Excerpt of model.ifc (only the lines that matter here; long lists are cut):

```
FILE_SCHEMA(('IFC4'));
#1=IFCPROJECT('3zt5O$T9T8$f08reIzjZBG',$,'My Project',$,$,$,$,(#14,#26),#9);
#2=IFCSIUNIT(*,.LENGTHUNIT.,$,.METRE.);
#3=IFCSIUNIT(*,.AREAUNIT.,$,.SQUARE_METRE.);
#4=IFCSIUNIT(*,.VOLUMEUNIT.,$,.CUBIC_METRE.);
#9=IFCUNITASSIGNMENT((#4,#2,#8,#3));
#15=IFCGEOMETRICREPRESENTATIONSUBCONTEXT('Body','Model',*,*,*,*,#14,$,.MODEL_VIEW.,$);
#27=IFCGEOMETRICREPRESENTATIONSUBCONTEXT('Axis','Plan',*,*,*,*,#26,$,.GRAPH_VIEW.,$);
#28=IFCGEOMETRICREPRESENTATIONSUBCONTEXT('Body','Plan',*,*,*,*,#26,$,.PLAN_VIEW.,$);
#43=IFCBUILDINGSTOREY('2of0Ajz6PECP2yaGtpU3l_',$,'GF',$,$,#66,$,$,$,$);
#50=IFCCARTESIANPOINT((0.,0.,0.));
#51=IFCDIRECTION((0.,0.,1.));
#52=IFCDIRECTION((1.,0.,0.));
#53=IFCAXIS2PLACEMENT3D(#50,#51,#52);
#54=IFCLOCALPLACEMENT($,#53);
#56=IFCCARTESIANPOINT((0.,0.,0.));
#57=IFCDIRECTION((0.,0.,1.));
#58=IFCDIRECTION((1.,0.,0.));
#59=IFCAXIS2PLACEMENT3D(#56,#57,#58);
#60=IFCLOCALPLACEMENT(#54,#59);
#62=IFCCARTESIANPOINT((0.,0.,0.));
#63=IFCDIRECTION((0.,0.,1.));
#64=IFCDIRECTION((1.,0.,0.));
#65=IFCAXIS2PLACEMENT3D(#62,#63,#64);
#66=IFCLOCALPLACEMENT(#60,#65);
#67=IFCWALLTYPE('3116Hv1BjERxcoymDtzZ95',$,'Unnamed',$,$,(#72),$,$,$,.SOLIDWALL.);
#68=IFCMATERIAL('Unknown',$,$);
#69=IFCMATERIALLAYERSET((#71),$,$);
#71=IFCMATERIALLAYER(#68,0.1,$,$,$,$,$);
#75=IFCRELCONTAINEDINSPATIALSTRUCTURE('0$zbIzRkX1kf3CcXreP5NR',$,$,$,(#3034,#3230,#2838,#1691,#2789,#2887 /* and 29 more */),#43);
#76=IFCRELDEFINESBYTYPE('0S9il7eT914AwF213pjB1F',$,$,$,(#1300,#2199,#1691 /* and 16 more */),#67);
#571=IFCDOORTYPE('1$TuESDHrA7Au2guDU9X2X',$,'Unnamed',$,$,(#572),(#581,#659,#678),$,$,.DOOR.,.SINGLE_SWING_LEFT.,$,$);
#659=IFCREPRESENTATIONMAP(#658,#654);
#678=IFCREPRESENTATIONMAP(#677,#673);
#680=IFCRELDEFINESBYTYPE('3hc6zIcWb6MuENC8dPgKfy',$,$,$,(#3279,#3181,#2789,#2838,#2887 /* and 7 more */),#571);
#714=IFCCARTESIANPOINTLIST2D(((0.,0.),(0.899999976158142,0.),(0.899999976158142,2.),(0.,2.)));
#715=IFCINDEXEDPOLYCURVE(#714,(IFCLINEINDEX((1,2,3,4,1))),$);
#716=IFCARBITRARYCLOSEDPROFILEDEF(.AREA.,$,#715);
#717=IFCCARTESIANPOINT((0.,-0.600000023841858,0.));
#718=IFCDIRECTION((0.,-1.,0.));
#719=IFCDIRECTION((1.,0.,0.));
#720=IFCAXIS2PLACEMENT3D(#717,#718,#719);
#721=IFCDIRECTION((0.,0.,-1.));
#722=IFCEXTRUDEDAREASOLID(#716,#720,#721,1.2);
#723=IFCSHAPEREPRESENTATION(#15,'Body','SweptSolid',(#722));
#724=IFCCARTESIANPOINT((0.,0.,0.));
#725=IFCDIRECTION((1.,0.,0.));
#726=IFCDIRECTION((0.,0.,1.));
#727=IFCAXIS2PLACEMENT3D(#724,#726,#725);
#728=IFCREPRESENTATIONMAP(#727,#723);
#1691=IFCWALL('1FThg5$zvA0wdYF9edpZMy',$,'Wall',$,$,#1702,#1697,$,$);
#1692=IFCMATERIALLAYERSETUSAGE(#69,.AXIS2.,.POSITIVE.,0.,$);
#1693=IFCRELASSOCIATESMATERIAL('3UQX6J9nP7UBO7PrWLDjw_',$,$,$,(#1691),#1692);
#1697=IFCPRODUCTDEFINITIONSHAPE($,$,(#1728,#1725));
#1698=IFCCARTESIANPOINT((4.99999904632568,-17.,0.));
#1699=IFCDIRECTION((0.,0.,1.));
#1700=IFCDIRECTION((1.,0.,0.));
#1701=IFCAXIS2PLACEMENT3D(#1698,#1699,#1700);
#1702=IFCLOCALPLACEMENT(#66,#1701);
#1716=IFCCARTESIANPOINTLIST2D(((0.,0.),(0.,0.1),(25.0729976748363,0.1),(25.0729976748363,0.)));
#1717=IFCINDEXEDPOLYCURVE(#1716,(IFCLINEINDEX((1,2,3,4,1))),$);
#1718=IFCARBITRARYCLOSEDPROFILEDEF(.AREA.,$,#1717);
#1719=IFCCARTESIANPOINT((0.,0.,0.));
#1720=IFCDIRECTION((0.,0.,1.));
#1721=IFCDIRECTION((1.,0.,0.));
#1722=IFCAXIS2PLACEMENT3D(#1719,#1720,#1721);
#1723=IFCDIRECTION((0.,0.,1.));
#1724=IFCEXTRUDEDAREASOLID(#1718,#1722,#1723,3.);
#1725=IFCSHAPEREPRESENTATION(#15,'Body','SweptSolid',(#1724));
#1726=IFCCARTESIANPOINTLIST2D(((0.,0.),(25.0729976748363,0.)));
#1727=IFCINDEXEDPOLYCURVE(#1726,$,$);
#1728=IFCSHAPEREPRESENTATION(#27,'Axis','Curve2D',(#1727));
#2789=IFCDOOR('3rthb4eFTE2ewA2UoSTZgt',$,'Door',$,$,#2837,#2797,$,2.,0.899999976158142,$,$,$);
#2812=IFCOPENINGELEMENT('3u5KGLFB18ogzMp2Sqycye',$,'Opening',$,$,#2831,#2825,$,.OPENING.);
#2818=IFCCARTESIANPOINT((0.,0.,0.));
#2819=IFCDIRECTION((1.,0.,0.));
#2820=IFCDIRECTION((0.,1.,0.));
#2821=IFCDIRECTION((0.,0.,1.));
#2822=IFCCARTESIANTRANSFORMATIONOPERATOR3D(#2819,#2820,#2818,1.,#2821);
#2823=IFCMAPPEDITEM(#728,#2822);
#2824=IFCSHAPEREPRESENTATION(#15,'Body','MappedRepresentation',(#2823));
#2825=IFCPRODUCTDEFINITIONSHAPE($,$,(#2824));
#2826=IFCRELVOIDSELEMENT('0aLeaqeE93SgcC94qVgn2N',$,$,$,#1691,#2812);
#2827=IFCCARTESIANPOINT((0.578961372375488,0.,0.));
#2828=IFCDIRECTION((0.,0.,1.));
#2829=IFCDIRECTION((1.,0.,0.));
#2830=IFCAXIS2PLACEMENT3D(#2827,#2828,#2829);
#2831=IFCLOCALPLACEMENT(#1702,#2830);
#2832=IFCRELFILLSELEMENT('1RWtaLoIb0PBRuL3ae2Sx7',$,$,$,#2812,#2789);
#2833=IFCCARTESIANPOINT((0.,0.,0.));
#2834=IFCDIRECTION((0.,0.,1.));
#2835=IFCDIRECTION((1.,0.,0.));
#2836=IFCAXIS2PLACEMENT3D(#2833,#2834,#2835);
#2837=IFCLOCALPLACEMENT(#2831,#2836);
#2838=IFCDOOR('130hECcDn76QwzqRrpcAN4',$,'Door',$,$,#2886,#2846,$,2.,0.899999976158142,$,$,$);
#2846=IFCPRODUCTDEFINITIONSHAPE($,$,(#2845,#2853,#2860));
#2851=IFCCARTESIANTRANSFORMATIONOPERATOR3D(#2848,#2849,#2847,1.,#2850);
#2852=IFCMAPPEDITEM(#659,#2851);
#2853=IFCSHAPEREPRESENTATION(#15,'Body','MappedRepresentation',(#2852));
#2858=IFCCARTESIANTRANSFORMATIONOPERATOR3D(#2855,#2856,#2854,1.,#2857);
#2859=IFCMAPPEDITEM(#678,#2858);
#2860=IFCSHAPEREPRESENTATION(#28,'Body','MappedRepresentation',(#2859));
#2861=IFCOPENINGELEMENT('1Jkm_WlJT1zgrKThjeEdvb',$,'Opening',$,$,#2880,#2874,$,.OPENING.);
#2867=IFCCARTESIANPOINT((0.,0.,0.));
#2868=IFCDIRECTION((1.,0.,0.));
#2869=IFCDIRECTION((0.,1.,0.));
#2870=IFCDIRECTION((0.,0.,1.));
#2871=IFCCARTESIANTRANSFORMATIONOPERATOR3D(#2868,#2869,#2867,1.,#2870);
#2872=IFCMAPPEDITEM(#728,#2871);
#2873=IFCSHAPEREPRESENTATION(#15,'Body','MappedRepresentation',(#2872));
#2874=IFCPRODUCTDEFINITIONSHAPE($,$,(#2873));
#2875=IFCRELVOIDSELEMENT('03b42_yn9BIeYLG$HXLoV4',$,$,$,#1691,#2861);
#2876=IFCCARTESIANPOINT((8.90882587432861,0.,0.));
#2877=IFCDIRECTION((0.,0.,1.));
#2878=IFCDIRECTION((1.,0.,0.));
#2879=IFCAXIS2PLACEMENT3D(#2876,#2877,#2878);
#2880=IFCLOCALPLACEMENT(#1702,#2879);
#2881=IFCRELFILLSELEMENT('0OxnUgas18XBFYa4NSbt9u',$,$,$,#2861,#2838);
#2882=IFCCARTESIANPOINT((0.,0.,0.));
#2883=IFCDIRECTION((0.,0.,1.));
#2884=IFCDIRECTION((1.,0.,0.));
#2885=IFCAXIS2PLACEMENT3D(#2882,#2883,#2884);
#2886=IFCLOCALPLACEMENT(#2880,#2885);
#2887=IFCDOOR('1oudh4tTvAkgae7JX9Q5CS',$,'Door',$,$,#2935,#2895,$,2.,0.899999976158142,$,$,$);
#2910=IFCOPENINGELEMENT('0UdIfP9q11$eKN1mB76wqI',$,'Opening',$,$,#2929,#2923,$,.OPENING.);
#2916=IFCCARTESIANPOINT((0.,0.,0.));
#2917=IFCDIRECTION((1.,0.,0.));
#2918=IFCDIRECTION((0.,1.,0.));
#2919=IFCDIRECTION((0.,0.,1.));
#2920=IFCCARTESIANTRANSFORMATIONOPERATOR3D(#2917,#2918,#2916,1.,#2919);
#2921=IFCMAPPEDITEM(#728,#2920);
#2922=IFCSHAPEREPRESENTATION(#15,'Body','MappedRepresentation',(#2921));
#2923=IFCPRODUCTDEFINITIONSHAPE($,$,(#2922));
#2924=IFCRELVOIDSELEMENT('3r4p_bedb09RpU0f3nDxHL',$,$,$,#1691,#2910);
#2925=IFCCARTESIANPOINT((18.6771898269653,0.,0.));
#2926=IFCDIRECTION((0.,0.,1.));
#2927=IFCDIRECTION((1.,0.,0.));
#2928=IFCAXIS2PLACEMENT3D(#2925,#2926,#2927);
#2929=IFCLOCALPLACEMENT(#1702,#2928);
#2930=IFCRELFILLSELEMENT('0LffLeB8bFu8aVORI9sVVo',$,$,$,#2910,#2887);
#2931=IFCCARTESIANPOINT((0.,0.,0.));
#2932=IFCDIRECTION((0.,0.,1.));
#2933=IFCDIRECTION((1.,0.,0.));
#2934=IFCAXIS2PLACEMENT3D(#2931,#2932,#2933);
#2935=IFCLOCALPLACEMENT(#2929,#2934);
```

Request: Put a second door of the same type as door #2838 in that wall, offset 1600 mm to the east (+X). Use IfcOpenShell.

```python
import ifcopenshell
import ifcopenshell.api.feature
import ifcopenshell.api.geometry
import ifcopenshell.api.root
import ifcopenshell.geom
import ifcopenshell.util.element
import ifcopenshell.util.placement
import ifcopenshell.util.shape

model = ifcopenshell.open("model.ifc")
settings = ifcopenshell.geom.settings()


def volume(element):
    """Net volume in cubic metres, openings subtracted."""
    shape = ifcopenshell.geom.create_shape(settings, element)
    return ifcopenshell.util.shape.get_volume(shape.geometry)


door = model.by_guid("130hECcDn76QwzqRrpcAN4")
opening = door.FillsVoids[0].RelatingOpeningElement
wall = opening.VoidsElements[0].RelatingBuildingElement
before = volume(wall)
shift = ifcopenshell.util.placement.get_local_placement(wall.ObjectPlacement)[:3, 0] * 1.6

# copy_class copies the void relationship, type, container and properties, but no geometry.
new_opening = ifcopenshell.api.root.copy_class(model, product=opening)
new_opening.Representation = ifcopenshell.util.element.copy_deep(
    model, opening.Representation, exclude=["IfcGeometricRepresentationContext", "IfcRepresentationMap"]
)
new_door = ifcopenshell.api.root.copy_class(model, product=door)
new_door.Representation = ifcopenshell.util.element.copy_deep(
    model, door.Representation, exclude=["IfcGeometricRepresentationContext", "IfcRepresentationMap"]
)
ifcopenshell.api.feature.add_filling(model, opening=new_opening, element=new_door)

for old, new in ((opening, new_opening), (door, new_door)):
    matrix = ifcopenshell.util.placement.get_local_placement(old.ObjectPlacement)
    matrix[:3, 3] += shift
    ifcopenshell.api.geometry.edit_object_placement(model, product=new, matrix=matrix, is_si=False)

after = volume(wall)

print(f"wall volume {before:.3f} -> {after:.3f} m3")

model.write("model-out.ifc")
```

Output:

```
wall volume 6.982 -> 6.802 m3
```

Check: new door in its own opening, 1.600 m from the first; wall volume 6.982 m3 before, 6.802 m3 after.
